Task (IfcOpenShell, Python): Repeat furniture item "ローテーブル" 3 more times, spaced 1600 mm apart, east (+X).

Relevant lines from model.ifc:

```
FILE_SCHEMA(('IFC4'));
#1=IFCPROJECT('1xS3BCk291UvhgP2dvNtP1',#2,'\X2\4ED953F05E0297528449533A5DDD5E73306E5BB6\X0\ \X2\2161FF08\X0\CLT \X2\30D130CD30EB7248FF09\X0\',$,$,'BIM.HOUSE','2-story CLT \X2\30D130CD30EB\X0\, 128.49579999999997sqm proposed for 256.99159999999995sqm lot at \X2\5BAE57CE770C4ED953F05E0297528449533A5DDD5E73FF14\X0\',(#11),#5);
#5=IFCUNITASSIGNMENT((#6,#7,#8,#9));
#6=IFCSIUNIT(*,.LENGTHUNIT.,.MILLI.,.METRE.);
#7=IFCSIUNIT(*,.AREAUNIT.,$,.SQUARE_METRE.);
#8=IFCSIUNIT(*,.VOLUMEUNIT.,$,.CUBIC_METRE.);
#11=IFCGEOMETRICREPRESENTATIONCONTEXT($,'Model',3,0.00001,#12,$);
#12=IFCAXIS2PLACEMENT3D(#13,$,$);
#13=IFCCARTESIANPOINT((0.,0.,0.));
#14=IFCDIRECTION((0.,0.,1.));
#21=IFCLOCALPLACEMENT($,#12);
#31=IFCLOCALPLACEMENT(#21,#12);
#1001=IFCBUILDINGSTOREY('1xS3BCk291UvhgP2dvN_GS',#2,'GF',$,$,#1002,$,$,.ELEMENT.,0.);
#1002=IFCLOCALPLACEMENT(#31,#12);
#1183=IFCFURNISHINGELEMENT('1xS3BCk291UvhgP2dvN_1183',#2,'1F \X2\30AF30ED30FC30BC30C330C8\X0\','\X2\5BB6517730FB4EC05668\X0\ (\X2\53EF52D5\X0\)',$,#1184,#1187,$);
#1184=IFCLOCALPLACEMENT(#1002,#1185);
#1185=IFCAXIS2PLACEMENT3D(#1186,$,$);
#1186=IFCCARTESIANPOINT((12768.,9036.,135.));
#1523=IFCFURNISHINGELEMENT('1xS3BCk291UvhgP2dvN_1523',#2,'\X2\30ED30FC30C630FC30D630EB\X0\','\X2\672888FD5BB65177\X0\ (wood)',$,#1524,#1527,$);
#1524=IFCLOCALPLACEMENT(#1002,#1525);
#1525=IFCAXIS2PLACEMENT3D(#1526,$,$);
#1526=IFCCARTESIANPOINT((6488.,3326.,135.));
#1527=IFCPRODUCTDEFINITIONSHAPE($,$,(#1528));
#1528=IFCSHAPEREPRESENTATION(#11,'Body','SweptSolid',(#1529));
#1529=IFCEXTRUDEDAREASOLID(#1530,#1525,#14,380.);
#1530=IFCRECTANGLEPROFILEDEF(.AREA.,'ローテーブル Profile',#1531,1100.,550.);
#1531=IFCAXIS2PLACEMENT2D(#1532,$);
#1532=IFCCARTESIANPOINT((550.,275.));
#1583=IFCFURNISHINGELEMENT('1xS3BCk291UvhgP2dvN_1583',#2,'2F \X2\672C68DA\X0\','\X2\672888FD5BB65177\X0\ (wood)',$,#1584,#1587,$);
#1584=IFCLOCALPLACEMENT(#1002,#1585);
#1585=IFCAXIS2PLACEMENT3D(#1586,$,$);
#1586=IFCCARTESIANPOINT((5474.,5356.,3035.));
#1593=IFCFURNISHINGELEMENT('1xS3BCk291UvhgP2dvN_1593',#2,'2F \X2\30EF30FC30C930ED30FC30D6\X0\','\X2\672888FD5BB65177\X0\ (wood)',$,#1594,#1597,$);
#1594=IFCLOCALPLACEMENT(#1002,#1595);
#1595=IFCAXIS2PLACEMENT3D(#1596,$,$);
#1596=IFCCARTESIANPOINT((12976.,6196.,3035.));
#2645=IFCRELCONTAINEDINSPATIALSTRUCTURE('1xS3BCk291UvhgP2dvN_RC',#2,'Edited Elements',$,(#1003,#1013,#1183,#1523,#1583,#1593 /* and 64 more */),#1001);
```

```python
import numpy as np
import ifcopenshell
import ifcopenshell.api.geometry
import ifcopenshell.api.root
import ifcopenshell.util.element
import ifcopenshell.util.placement

model = ifcopenshell.open("model.ifc")


def reuse_history(source, copy):
    """copy_class also copies each property set's owner history, people and application; keep the originals."""
    for rel in copy.IsDefinedBy:
        if rel.is_a("IfcRelDefinesByProperties") and (history := rel.RelatingPropertyDefinition.OwnerHistory):
            rel.RelatingPropertyDefinition.OwnerHistory = source.OwnerHistory
            ifcopenshell.util.element.remove_deep2(model, history)


source = model.by_guid("1xS3BCk291UvhgP2dvN_1523")
base = ifcopenshell.util.placement.get_local_placement(source.ObjectPlacement)
step = np.array([1.0, 0.0, 0.0]) * 1600.0

for i in range(1, 4):
    copy = ifcopenshell.api.root.copy_class(model, product=source)
    copy.Representation = ifcopenshell.util.element.copy_deep(
        model, source.Representation, exclude=["IfcGeometricRepresentationContext", "IfcRepresentationMap"]
    )
    reuse_history(source, copy)
    matrix = base.copy()
    matrix[:3, 3] += i * step
    print("added at", matrix[:3, 3].round(3) + 0.0)
    ifcopenshell.api.geometry.edit_object_placement(model, product=copy, matrix=matrix, is_si=False)

model.write("model_rev.ifc")
```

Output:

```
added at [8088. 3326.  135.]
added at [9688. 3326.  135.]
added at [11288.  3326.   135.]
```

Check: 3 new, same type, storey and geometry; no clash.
